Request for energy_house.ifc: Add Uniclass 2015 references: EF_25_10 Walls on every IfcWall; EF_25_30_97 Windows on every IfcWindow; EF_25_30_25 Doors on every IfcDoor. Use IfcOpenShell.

First a look at what the model holds.

```python
import ifcopenshell

model = ifcopenshell.open("energy_house.ifc")
print(model.schema)
print("classifications:", [c.Name for c in model.by_type("IfcClassification")])
for ifc_class in ("IfcDoor", "IfcRoof", "IfcStair", "IfcWall", "IfcWindow"):
    print(ifc_class, len(model.by_type(ifc_class)))
```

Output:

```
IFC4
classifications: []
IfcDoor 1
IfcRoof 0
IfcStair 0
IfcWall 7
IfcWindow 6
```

```python
import ifcopenshell
import ifcopenshell.api.classification

model = ifcopenshell.open("energy_house.ifc")

system = ifcopenshell.api.classification.add_classification(model, classification="Uniclass 2015")

codes = {
    "IfcWall": ("EF_25_10", "Walls"),
    "IfcWindow": ("EF_25_30_97", "Windows"),
    "IfcDoor": ("EF_25_30_25", "Doors"),
}
for ifc_class, (code, name) in codes.items():
    products = model.by_type(ifc_class)
    ifcopenshell.api.classification.add_reference(
        model, products=products, classification=system, identification=code, name=name
    )
    print(code, len(products))

model.write("energy_house_edited.ifc")
```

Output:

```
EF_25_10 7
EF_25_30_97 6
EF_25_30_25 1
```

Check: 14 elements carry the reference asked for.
